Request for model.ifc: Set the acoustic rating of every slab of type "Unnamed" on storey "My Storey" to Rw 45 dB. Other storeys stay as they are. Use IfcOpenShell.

First a look at what the model holds.

```python
import ifcopenshell
import ifcopenshell.util.element

model = ifcopenshell.open("model.ifc")
print(model.schema)
storey = next(s for s in model.by_type("IfcBuildingStorey") if s.Name == "My Storey")
slabs = [e for e in ifcopenshell.util.element.get_decomposition(storey) if e.is_a("IfcSlab")]
seen = {}
for e in slabs:
    element_type = ifcopenshell.util.element.get_type(e)
    key = (element_type.Name if element_type != e and element_type else None, ifcopenshell.util.element.get_pset(e, "Pset_SlabCommon", "AcousticRating"))
    seen[key] = seen.get(key, 0) + 1
for (name, value), count in sorted(seen.items(), key=str):
    print(count, "x", name, "|", value)
```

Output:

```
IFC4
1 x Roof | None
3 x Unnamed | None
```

```python
import ifcopenshell
import ifcopenshell.api.pset
import ifcopenshell.util.element

model = ifcopenshell.open("model.ifc")

storey = next(s for s in model.by_type("IfcBuildingStorey") if s.Name == "My Storey")
slabs = [e for e in ifcopenshell.util.element.get_decomposition(storey) if e.is_a("IfcSlab")]

count = 0
for e in slabs:
    element_type = ifcopenshell.util.element.get_type(e)
    if element_type in (None, e) or element_type.Name != "Unnamed":
        continue
    # add_pset returns the element's existing set when there is one.
    pset = ifcopenshell.api.pset.add_pset(model, product=e, name="Pset_SlabCommon")
    ifcopenshell.api.pset.edit_pset(model, pset=pset, properties={"AcousticRating": "Rw 45 dB"})
    count += 1

print(count, "slabs updated")

model.write("model_rev.ifc")
```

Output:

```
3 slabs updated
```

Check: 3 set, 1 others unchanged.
